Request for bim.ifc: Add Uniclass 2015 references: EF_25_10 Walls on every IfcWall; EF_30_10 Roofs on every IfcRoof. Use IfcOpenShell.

First a look at what the model holds.

```python
import ifcopenshell

model = ifcopenshell.open("bim.ifc")
print(model.schema)
print("classifications:", [c.Name for c in model.by_type("IfcClassification")])
for ifc_class in ("IfcDoor", "IfcRoof", "IfcStair", "IfcWall", "IfcWindow"):
    print(ifc_class, len(model.by_type(ifc_class)))
```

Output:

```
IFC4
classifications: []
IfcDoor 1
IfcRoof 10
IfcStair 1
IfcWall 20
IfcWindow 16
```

```python
import ifcopenshell
import ifcopenshell.api.classification

model = ifcopenshell.open("bim.ifc")

system = ifcopenshell.api.classification.add_classification(model, classification="Uniclass 2015")

codes = {
    "IfcWall": ("EF_25_10", "Walls"),
    "IfcRoof": ("EF_30_10", "Roofs"),
}
for ifc_class, (code, name) in codes.items():
    products = model.by_type(ifc_class)
    ifcopenshell.api.classification.add_reference(
        model, products=products, classification=system, identification=code, name=name
    )
    print(code, len(products))

model.write("bim_rev.ifc")
```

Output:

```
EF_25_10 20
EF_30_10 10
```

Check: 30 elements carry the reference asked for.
